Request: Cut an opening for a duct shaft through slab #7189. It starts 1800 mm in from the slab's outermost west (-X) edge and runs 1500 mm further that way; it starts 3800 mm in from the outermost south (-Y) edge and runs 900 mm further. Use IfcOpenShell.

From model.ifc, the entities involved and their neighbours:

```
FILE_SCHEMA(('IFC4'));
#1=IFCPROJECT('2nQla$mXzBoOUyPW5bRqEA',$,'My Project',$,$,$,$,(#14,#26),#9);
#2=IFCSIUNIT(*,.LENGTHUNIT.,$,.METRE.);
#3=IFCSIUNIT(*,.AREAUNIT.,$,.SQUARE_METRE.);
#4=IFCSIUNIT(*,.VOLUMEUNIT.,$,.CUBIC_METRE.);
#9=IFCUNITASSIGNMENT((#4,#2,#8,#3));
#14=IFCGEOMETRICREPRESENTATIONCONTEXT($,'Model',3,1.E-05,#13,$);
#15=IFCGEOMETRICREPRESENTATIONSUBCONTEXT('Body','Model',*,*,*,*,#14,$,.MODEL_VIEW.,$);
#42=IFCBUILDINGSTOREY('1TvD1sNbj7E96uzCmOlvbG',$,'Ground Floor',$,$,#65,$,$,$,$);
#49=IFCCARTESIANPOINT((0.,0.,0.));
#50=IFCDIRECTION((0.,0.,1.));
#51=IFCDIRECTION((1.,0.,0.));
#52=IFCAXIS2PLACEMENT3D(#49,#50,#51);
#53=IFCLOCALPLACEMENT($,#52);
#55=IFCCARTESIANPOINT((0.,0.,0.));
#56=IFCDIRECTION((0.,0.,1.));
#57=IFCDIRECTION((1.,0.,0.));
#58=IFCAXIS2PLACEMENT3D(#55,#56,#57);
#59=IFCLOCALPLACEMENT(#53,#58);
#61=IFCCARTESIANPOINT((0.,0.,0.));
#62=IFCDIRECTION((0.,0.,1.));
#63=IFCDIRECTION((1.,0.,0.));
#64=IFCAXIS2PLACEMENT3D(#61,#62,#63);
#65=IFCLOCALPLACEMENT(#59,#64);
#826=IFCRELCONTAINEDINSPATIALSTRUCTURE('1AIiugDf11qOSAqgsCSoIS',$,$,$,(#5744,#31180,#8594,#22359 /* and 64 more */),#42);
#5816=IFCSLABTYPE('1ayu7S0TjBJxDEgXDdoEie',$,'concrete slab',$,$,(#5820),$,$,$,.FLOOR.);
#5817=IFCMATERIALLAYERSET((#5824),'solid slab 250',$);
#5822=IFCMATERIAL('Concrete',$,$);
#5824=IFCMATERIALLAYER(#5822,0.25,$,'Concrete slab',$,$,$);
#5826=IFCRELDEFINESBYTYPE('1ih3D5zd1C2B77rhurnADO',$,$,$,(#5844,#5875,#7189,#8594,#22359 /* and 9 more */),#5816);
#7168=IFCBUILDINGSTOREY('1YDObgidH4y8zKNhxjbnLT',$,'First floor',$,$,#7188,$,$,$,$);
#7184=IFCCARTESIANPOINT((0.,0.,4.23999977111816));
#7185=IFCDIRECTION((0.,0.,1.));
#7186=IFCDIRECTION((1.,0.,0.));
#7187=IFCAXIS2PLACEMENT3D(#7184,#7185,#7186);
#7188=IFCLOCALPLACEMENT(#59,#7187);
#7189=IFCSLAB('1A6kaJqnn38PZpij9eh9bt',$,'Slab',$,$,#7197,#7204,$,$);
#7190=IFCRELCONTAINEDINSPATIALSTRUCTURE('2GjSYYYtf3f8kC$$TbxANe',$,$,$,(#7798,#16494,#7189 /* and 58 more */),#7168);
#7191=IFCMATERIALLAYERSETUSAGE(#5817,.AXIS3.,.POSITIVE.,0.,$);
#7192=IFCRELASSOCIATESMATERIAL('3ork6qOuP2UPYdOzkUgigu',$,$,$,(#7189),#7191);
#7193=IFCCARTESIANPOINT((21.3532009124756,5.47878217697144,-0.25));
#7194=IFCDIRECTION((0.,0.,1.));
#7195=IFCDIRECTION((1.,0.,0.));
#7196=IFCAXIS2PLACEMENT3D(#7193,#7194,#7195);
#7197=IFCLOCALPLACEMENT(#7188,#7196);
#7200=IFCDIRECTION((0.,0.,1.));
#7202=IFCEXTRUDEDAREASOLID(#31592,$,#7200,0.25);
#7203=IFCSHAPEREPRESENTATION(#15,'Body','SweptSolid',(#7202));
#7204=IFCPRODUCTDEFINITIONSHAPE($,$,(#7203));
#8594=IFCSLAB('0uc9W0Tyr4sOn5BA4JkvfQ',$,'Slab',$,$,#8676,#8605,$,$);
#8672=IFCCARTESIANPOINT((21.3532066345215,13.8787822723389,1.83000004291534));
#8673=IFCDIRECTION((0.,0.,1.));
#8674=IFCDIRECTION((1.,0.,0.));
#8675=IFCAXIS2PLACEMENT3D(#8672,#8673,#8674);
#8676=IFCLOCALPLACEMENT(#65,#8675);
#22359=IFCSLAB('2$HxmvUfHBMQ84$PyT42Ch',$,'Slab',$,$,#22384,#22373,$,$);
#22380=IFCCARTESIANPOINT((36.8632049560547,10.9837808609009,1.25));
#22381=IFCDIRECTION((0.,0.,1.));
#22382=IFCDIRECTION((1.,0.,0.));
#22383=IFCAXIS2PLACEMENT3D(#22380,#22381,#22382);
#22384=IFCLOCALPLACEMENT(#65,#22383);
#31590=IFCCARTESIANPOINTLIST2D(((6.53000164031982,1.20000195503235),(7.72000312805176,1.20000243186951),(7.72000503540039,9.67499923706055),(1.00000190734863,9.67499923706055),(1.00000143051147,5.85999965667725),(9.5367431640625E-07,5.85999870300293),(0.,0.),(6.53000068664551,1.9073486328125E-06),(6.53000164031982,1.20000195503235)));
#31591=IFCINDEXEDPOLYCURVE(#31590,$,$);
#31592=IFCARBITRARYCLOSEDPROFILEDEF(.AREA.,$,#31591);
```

```python
import numpy as np
import ifcopenshell
import ifcopenshell.api.feature
import ifcopenshell.api.geometry
import ifcopenshell.api.root
import ifcopenshell.geom
import ifcopenshell.util.placement
import ifcopenshell.util.representation
import ifcopenshell.util.shape
import ifcopenshell.util.unit

model = ifcopenshell.open("model.ifc")
unit_scale = ifcopenshell.util.unit.calculate_unit_scale(model)
settings = ifcopenshell.geom.settings()


def volume(element):
    """Net volume in cubic metres, openings subtracted."""
    shape = ifcopenshell.geom.create_shape(settings, element)
    return ifcopenshell.util.shape.get_volume(shape.geometry)


slab = model.by_guid("1A6kaJqnn38PZpij9eh9bt")
before = volume(slab)

# Extent in the slab's own axes, in metres. The edges named are its -X and -Y sides.
slab_shape = ifcopenshell.geom.create_shape(settings, slab)
vertices = ifcopenshell.util.shape.get_vertices(slab_shape.geometry)
x_min, y_min, bottom = vertices.min(axis=0)
top = vertices[:, 2].max()

opening = ifcopenshell.api.root.create_entity(model, ifc_class="IfcOpeningElement", name="Duct shaft opening", predefined_type="OPENING")
context = ifcopenshell.util.representation.get_context(model, "Model", "Body", "MODEL_VIEW")
width, depth = 1.5, 0.9
outline = [(0.0, 0.0), (width, 0.0), (width, depth), (0.0, depth), (0.0, 0.0)]
# Overshoot both faces by 50 mm so the cut is clean.
shape = ifcopenshell.api.geometry.add_slab_representation(
    model, context=context, depth=top - bottom + 0.1, polyline=outline
)
ifcopenshell.api.geometry.assign_representation(model, product=opening, representation=shape)

matrix = ifcopenshell.util.placement.get_local_placement(slab.ObjectPlacement)
matrix[:, 3] = matrix @ np.append(np.array([x_min + 1.8, y_min + 3.8, bottom - 0.05]) / unit_scale, 1.0)
ifcopenshell.api.geometry.edit_object_placement(model, product=opening, matrix=matrix, is_si=False)
ifcopenshell.api.feature.add_feature(model, feature=opening, element=slab)

after = volume(slab)

print(f"slab volume {before:.3f} -> {after:.3f} m3")

model.write("model_v2.ifc")
```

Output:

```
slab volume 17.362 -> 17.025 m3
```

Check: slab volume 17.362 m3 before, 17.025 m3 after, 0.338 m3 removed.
